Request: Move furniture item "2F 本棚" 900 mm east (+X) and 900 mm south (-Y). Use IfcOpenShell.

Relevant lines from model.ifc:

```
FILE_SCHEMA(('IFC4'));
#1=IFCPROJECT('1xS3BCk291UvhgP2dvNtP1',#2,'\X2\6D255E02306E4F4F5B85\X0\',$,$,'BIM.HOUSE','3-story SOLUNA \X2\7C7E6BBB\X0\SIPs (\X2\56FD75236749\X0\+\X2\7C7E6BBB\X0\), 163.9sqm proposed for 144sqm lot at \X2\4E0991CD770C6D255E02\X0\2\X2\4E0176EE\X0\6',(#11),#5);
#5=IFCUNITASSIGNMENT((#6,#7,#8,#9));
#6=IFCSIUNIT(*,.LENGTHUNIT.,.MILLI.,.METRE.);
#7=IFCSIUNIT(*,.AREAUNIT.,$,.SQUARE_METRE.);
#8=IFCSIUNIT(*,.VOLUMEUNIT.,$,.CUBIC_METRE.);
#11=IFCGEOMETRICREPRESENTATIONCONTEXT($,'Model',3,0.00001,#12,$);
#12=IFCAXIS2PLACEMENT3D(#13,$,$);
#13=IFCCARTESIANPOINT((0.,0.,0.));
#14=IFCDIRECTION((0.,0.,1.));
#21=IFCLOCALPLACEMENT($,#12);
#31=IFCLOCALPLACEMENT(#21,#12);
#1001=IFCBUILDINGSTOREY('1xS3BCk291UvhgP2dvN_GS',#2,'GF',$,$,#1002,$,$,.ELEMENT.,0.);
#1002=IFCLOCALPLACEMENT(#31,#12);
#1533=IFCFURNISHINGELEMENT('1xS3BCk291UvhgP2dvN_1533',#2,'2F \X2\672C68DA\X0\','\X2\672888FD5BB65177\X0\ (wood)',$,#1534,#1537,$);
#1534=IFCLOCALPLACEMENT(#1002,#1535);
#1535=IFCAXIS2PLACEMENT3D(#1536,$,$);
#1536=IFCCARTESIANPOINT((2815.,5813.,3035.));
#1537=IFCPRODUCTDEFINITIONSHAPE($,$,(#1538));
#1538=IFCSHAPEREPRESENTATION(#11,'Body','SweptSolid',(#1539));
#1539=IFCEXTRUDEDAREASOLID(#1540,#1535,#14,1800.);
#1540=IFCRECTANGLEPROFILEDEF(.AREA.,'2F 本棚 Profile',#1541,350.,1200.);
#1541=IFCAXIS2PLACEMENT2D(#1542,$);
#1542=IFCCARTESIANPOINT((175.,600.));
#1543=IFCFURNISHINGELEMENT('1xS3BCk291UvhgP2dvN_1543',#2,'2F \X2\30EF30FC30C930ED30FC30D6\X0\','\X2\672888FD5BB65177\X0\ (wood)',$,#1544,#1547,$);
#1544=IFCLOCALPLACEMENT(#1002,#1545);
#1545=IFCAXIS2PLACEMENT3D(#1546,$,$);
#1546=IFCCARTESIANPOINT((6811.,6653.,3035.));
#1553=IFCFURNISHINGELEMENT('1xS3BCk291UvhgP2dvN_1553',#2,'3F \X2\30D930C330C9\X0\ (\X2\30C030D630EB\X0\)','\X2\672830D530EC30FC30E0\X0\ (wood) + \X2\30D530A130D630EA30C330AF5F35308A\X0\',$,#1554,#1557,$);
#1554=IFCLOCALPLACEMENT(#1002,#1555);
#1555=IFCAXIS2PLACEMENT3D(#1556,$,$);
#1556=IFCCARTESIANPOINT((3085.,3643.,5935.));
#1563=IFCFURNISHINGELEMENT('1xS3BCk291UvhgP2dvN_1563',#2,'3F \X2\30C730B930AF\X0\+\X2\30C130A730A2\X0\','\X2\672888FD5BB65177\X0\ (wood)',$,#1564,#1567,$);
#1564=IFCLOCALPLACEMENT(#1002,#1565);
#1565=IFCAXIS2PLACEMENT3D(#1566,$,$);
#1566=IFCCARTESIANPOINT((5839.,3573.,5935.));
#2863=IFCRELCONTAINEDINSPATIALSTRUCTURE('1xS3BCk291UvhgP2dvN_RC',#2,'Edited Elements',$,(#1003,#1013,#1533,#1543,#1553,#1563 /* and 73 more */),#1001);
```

```python
import ifcopenshell
import ifcopenshell.api.geometry
import ifcopenshell.util.placement
import ifcopenshell.util.unit

model = ifcopenshell.open("model.ifc")
unit_scale = ifcopenshell.util.unit.calculate_unit_scale(model)

item = model.by_guid("1xS3BCk291UvhgP2dvN_1533")
matrix = ifcopenshell.util.placement.get_local_placement(item.ObjectPlacement)
matrix[0, 3] += 0.9 / unit_scale
matrix[1, 3] -= 0.9 / unit_scale
ifcopenshell.api.geometry.edit_object_placement(model, product=item, matrix=matrix, is_si=False)

print(ifcopenshell.util.placement.get_local_placement(item.ObjectPlacement).round(3) + 0.0)

model.write("model_edited.ifc")
```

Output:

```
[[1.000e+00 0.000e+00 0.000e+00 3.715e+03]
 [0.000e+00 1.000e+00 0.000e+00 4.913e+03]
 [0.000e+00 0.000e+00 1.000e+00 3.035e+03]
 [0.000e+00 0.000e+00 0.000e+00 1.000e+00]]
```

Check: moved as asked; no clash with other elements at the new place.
